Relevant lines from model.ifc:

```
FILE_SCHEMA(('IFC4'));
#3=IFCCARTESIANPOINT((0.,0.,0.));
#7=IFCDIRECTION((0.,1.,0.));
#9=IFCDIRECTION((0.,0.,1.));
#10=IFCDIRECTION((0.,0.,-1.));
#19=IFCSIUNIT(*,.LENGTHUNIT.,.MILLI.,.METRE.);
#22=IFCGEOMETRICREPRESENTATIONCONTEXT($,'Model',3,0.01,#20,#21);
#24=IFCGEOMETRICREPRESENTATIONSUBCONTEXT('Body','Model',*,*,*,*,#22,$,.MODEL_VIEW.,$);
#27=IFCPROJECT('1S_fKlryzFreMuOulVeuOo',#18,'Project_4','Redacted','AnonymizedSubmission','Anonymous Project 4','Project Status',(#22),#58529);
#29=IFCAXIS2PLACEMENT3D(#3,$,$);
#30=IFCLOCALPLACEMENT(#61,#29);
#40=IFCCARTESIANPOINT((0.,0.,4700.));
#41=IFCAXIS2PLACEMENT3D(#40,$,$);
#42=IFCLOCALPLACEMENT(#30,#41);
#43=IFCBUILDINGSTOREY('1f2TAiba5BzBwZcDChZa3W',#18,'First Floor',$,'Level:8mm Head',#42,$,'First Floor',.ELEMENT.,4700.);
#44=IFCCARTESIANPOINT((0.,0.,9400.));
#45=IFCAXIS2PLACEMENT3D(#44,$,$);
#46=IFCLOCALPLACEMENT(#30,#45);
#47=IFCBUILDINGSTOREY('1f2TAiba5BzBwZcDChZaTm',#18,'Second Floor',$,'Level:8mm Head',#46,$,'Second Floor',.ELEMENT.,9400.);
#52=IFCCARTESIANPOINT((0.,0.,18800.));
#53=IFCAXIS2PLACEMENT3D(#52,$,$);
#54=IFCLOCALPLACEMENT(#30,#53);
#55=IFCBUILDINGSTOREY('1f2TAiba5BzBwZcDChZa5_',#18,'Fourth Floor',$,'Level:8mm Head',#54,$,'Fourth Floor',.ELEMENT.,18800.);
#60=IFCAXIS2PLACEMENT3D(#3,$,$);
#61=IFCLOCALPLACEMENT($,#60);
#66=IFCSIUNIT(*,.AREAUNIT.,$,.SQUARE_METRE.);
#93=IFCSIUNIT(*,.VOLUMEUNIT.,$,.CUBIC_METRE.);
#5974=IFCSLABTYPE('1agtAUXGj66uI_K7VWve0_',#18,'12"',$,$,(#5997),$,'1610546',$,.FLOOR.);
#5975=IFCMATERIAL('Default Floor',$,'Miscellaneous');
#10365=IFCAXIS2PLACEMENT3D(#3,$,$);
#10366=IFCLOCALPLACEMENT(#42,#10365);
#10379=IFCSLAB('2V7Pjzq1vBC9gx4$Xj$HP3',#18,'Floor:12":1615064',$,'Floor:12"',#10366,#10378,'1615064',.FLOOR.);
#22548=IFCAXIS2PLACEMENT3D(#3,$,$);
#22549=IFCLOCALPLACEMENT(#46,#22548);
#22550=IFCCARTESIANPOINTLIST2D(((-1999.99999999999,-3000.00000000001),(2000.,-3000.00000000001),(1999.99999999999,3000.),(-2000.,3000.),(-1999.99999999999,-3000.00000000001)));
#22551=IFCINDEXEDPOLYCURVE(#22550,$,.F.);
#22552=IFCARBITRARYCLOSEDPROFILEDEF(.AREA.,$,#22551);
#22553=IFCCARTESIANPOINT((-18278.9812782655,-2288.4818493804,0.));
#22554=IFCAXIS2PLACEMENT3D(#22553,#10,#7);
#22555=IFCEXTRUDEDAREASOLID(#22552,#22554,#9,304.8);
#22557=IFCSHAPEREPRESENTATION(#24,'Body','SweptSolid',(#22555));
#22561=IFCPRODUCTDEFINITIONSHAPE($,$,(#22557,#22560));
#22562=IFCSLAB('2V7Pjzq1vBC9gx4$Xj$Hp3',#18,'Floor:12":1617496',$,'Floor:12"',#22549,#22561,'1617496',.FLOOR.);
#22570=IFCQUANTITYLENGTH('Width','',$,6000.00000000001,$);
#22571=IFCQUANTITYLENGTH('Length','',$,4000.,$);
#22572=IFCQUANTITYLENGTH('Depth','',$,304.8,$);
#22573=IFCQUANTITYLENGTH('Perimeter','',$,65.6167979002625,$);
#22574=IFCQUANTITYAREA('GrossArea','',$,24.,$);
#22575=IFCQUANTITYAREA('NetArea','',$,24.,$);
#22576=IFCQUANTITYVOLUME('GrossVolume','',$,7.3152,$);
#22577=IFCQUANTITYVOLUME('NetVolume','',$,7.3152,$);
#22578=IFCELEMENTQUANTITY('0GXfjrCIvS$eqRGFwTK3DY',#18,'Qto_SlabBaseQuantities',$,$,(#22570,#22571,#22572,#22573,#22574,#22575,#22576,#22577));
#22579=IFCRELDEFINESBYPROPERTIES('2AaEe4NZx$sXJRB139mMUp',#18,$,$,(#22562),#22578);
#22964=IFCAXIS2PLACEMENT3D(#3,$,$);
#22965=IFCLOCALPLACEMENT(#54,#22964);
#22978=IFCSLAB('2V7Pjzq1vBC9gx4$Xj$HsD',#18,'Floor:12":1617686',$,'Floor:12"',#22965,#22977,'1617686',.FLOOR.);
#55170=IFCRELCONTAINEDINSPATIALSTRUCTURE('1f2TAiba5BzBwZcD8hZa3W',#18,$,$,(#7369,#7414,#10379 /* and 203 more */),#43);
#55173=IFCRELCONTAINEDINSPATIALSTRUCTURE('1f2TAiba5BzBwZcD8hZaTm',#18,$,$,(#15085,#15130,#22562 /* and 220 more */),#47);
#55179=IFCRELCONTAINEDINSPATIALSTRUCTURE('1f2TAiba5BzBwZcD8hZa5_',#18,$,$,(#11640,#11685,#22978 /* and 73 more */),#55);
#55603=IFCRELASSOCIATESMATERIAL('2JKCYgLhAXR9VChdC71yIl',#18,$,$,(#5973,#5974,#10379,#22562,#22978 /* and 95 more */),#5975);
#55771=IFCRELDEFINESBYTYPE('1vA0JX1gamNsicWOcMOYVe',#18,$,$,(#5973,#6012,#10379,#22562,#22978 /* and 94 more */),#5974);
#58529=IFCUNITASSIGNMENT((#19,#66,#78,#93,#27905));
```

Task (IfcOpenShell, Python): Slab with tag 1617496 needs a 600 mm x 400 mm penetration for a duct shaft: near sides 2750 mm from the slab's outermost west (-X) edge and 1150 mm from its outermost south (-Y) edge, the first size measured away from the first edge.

```python
import numpy as np
import ifcopenshell
import ifcopenshell.api.feature
import ifcopenshell.api.geometry
import ifcopenshell.api.pset
import ifcopenshell.api.root
import ifcopenshell.geom
import ifcopenshell.util.element
import ifcopenshell.util.placement
import ifcopenshell.util.representation
import ifcopenshell.util.shape
import ifcopenshell.util.unit

model = ifcopenshell.open("model.ifc")
unit_scale = ifcopenshell.util.unit.calculate_unit_scale(model)
area_scale = ifcopenshell.util.unit.calculate_unit_scale(model, "AREAUNIT")
volume_scale = ifcopenshell.util.unit.calculate_unit_scale(model, "VOLUMEUNIT")
settings = ifcopenshell.geom.settings()


def volume(element):
    """Net volume in cubic metres, openings subtracted."""
    shape = ifcopenshell.geom.create_shape(settings, element)
    return ifcopenshell.util.shape.get_volume(shape.geometry)


slab = model.by_guid("2V7Pjzq1vBC9gx4$Xj$Hp3")
before = volume(slab)

# Extent in the slab's own axes, in metres. The edges named are its -X and -Y sides.
slab_shape = ifcopenshell.geom.create_shape(settings, slab)
vertices = ifcopenshell.util.shape.get_vertices(slab_shape.geometry)
x_min, y_min, bottom = vertices.min(axis=0)
top = vertices[:, 2].max()

opening = ifcopenshell.api.root.create_entity(model, ifc_class="IfcOpeningElement", name="Duct shaft opening", predefined_type="OPENING")
context = ifcopenshell.util.representation.get_context(model, "Model", "Body", "MODEL_VIEW")
width, depth = 0.6, 0.4
outline = [(0.0, 0.0), (width, 0.0), (width, depth), (0.0, depth), (0.0, 0.0)]
# Overshoot both faces by 50 mm so the cut is clean.
shape = ifcopenshell.api.geometry.add_slab_representation(
    model, context=context, depth=top - bottom + 0.1, polyline=outline
)
ifcopenshell.api.geometry.assign_representation(model, product=opening, representation=shape)

matrix = ifcopenshell.util.placement.get_local_placement(slab.ObjectPlacement)
matrix[:, 3] = matrix @ np.append(np.array([x_min + 2.75, y_min + 1.15, bottom - 0.05]) / unit_scale, 1.0)
ifcopenshell.api.geometry.edit_object_placement(model, product=opening, matrix=matrix, is_si=False)
ifcopenshell.api.feature.add_feature(model, feature=opening, element=slab)

after = volume(slab)

# Update the slab's stored quantities.
qto = model.by_id(ifcopenshell.util.element.get_pset(slab, "Qto_SlabBaseQuantities", should_inherit=False)["id"])
ifcopenshell.api.pset.edit_qto(model, qto=qto, properties={
    "NetArea": after / (top - bottom) / area_scale,
    "NetVolume": after / volume_scale,
})

print(f"slab volume {before:.3f} -> {after:.3f} m3")

model.write("model_v2.ifc")
```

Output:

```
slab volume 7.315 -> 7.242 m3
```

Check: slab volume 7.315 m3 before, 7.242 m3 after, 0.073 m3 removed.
